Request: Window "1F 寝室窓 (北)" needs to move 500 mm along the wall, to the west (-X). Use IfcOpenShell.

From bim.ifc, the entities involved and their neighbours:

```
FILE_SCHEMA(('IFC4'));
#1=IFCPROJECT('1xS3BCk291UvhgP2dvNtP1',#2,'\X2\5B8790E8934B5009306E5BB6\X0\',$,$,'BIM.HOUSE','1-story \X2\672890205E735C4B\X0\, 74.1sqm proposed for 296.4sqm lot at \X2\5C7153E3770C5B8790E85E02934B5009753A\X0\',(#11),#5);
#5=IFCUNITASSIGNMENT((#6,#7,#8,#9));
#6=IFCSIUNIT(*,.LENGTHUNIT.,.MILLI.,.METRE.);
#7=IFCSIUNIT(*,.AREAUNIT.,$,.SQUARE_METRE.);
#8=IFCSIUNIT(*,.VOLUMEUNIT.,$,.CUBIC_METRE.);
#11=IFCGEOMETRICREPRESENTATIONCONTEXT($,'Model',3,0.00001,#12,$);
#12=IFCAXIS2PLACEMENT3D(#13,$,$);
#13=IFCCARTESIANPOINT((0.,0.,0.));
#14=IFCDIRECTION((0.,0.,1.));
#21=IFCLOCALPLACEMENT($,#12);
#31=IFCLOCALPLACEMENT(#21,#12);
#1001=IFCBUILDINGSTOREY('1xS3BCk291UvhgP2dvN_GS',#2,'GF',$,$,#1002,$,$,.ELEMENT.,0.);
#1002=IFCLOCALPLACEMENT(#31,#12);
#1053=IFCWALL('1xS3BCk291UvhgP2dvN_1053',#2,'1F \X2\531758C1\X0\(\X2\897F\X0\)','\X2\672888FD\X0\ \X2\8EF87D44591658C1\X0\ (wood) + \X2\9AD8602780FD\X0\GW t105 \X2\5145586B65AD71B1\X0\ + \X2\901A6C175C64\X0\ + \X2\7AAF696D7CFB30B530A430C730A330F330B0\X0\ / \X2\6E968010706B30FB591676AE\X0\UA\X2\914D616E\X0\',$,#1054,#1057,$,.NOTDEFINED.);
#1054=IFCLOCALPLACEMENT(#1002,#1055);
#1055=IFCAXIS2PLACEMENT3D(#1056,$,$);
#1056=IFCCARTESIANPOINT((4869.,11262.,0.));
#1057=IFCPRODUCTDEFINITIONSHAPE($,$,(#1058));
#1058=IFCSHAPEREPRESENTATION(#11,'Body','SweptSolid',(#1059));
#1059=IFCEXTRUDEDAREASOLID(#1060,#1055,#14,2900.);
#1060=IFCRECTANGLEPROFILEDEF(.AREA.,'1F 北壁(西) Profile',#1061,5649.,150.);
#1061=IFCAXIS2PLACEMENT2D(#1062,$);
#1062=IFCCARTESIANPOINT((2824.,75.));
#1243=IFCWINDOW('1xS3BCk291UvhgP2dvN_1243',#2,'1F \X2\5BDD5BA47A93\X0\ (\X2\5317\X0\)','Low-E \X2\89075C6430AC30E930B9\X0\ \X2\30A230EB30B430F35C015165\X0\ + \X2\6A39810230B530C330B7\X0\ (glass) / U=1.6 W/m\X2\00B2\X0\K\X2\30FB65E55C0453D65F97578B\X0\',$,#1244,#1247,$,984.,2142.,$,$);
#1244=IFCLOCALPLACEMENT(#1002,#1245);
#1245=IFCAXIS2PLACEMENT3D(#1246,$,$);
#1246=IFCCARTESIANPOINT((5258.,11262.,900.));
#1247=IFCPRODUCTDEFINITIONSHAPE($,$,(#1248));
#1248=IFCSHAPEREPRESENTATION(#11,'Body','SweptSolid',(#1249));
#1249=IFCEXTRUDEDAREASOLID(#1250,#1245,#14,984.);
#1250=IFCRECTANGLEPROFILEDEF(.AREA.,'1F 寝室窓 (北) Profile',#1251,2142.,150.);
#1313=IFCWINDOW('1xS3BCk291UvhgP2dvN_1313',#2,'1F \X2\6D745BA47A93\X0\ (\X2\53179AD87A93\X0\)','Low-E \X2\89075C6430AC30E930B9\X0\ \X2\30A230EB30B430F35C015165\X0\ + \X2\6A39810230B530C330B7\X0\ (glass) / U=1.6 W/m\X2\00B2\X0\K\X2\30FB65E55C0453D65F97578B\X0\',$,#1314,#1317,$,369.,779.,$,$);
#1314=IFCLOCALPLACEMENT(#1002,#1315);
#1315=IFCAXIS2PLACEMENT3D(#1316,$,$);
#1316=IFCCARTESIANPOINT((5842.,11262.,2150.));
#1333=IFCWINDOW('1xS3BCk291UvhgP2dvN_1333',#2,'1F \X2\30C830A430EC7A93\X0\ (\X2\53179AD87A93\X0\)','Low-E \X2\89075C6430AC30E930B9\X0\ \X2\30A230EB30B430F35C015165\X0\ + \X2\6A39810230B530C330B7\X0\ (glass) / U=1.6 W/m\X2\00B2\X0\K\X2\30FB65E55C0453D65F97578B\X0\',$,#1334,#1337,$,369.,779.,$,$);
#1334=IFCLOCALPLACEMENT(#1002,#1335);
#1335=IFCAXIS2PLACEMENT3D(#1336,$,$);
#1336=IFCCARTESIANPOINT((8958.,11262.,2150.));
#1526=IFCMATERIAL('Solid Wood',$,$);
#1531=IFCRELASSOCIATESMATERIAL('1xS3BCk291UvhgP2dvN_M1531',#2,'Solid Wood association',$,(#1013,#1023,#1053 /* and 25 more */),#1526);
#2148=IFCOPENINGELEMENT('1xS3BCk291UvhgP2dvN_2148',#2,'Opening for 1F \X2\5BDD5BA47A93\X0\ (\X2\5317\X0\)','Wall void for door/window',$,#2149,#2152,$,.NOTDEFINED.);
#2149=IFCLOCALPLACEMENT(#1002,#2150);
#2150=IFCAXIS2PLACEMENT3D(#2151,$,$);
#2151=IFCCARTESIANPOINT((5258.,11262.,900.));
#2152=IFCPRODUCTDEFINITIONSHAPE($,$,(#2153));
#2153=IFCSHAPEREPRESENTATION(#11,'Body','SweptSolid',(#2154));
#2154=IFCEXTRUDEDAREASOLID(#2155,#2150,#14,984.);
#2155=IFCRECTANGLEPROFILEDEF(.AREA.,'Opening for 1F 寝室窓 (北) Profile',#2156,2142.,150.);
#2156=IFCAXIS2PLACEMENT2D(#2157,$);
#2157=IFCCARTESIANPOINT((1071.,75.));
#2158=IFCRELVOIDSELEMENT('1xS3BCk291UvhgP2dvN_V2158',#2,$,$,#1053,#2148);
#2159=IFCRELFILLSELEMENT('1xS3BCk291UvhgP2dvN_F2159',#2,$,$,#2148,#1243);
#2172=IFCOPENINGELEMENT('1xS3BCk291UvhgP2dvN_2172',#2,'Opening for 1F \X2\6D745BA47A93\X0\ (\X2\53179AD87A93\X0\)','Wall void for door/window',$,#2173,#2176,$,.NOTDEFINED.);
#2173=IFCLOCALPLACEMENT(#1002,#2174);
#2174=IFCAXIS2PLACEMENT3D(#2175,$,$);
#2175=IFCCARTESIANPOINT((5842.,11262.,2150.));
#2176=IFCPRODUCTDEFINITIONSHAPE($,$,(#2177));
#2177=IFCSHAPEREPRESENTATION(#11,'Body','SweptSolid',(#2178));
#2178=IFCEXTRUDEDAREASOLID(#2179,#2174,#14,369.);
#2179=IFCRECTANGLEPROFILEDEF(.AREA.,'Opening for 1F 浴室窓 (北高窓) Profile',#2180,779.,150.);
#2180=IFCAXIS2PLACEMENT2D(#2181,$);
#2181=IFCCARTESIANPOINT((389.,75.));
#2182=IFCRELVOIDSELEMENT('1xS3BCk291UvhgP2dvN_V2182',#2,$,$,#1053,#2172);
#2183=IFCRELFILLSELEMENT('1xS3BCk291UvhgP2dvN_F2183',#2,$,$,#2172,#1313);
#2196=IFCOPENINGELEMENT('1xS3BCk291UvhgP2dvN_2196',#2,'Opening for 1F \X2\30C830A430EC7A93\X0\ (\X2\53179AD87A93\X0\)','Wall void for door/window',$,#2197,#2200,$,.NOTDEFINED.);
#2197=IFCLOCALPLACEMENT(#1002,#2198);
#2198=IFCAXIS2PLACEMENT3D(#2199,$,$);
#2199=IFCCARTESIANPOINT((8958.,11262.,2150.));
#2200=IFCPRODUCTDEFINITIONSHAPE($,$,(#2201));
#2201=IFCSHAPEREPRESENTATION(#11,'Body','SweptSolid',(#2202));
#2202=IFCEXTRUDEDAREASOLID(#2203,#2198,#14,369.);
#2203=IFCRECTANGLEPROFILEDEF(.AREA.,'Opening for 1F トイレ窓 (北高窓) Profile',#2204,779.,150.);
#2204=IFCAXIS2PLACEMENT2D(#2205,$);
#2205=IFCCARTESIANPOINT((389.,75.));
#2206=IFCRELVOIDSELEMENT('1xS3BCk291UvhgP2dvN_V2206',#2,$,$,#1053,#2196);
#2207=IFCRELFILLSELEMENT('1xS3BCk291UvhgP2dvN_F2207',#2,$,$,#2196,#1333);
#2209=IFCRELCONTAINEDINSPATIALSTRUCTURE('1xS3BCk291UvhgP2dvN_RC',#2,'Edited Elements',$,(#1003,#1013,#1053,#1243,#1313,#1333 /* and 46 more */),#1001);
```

```python
import ifcopenshell
import ifcopenshell.api.geometry
import ifcopenshell.util.placement
import ifcopenshell.util.unit

model = ifcopenshell.open("bim.ifc")
unit_scale = ifcopenshell.util.unit.calculate_unit_scale(model)

window = model.by_id(1243)
opening = window.FillsVoids[0].RelatingOpeningElement
wall = opening.VoidsElements[0].RelatingBuildingElement

wall_matrix = ifcopenshell.util.placement.get_local_placement(wall.ObjectPlacement)
shift = wall_matrix[:3, 0] * -0.5 / unit_scale
before = ifcopenshell.util.placement.get_local_placement(window.ObjectPlacement)[:3, 3].copy()

# The window is not placed relative to its opening, so move both.
for product in (opening, window):
    matrix = ifcopenshell.util.placement.get_local_placement(product.ObjectPlacement)
    matrix[:3, 3] += shift
    ifcopenshell.api.geometry.edit_object_placement(model, product=product, matrix=matrix, is_si=False)

after = ifcopenshell.util.placement.get_local_placement(window.ObjectPlacement)[:3, 3]
print("window moved by", (after - before).round(3) + 0.0)

model.write("bim_updated.ifc")
```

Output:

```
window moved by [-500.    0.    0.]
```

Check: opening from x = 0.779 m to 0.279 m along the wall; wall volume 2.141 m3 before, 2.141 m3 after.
